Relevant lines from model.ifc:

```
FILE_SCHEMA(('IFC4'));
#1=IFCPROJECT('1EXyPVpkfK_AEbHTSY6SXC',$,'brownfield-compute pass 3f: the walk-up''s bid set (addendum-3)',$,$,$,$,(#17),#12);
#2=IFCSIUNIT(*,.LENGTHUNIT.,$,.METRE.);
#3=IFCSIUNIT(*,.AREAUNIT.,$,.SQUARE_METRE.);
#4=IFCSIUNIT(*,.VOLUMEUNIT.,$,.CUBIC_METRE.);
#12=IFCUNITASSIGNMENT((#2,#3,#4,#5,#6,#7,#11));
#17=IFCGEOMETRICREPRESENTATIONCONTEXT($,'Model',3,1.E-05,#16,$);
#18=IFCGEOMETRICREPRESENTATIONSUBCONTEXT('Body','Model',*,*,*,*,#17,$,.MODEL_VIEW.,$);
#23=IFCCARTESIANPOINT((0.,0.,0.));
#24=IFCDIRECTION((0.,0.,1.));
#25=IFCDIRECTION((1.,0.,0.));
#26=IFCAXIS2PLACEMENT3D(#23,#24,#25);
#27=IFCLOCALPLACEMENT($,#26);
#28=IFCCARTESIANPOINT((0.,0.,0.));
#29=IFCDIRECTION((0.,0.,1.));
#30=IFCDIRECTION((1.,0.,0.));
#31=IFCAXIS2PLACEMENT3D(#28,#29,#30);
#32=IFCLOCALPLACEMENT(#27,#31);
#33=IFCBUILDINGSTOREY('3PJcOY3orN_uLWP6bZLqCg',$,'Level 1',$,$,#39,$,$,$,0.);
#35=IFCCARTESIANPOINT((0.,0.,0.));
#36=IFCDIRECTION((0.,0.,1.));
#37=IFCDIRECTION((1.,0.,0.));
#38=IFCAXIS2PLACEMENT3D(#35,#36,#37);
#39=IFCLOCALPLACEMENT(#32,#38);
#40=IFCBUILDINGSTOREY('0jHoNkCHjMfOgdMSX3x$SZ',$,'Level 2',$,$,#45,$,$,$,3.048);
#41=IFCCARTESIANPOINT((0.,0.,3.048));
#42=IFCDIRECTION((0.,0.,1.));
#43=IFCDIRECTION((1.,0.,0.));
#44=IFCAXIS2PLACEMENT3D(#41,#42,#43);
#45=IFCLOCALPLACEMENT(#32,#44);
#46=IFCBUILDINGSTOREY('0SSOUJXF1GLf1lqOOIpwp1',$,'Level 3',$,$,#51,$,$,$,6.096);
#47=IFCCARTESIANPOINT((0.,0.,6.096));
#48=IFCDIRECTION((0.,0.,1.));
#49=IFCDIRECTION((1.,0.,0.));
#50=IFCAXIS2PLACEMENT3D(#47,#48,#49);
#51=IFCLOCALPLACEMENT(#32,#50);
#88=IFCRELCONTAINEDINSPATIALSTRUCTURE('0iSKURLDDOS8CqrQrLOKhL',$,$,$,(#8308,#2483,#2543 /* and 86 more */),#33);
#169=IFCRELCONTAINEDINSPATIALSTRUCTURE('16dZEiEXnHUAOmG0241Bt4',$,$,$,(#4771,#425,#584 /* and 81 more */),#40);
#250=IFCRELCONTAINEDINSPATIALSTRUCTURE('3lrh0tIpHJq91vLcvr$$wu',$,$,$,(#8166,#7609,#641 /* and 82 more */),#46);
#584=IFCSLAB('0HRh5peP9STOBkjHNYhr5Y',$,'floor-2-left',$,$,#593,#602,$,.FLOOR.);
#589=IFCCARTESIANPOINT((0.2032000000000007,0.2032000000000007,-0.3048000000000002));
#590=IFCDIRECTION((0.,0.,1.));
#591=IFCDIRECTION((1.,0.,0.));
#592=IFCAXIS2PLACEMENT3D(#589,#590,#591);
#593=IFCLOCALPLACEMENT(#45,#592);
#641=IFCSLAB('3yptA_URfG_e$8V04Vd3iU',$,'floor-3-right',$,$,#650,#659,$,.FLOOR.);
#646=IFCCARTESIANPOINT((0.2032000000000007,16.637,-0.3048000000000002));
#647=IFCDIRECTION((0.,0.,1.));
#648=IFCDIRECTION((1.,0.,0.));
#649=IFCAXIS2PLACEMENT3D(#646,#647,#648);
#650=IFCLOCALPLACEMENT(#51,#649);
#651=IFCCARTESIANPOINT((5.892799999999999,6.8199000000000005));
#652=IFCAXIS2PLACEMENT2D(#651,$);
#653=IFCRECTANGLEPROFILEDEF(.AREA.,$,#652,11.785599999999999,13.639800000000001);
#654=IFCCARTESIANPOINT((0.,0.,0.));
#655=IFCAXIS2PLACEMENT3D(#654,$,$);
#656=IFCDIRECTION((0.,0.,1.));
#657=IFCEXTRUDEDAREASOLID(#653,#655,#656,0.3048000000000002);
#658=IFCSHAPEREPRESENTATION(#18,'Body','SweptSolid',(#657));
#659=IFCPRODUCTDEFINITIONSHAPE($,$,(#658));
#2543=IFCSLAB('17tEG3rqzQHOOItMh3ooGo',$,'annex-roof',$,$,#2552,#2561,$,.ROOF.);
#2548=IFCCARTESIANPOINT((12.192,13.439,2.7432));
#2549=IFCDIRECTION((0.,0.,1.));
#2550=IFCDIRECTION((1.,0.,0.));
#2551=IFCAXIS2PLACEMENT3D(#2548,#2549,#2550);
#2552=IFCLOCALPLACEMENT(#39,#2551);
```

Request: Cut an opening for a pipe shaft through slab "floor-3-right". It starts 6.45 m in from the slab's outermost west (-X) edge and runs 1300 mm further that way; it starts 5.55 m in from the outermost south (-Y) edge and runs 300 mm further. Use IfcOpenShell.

```python
import numpy as np
import ifcopenshell
import ifcopenshell.api.feature
import ifcopenshell.api.geometry
import ifcopenshell.api.root
import ifcopenshell.geom
import ifcopenshell.util.placement
import ifcopenshell.util.representation
import ifcopenshell.util.shape
import ifcopenshell.util.unit

model = ifcopenshell.open("model.ifc")
unit_scale = ifcopenshell.util.unit.calculate_unit_scale(model)
settings = ifcopenshell.geom.settings()


def volume(element):
    """Net volume in cubic metres, openings subtracted."""
    shape = ifcopenshell.geom.create_shape(settings, element)
    return ifcopenshell.util.shape.get_volume(shape.geometry)


slab = model.by_guid("3yptA_URfG_e$8V04Vd3iU")
before = volume(slab)

# Extent in the slab's own axes, in metres. The edges named are its -X and -Y sides.
slab_shape = ifcopenshell.geom.create_shape(settings, slab)
vertices = ifcopenshell.util.shape.get_vertices(slab_shape.geometry)
x_min, y_min, bottom = vertices.min(axis=0)
top = vertices[:, 2].max()

opening = ifcopenshell.api.root.create_entity(model, ifc_class="IfcOpeningElement", name="Pipe shaft opening", predefined_type="OPENING")
context = ifcopenshell.util.representation.get_context(model, "Model", "Body", "MODEL_VIEW")
width, depth = 1.3, 0.3
outline = [(0.0, 0.0), (width, 0.0), (width, depth), (0.0, depth), (0.0, 0.0)]
# Overshoot both faces by 50 mm so the cut is clean.
shape = ifcopenshell.api.geometry.add_slab_representation(
    model, context=context, depth=top - bottom + 0.1, polyline=outline
)
ifcopenshell.api.geometry.assign_representation(model, product=opening, representation=shape)

matrix = ifcopenshell.util.placement.get_local_placement(slab.ObjectPlacement)
matrix[:, 3] = matrix @ np.append(np.array([x_min + 6.45, y_min + 5.55, bottom - 0.05]) / unit_scale, 1.0)
ifcopenshell.api.geometry.edit_object_placement(model, product=opening, matrix=matrix, is_si=False)
ifcopenshell.api.feature.add_feature(model, feature=opening, element=slab)

after = volume(slab)

print(f"slab volume {before:.3f} -> {after:.3f} m3")

model.write("model_edited.ifc")
```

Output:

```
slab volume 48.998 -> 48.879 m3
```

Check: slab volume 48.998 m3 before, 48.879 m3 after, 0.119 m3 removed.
